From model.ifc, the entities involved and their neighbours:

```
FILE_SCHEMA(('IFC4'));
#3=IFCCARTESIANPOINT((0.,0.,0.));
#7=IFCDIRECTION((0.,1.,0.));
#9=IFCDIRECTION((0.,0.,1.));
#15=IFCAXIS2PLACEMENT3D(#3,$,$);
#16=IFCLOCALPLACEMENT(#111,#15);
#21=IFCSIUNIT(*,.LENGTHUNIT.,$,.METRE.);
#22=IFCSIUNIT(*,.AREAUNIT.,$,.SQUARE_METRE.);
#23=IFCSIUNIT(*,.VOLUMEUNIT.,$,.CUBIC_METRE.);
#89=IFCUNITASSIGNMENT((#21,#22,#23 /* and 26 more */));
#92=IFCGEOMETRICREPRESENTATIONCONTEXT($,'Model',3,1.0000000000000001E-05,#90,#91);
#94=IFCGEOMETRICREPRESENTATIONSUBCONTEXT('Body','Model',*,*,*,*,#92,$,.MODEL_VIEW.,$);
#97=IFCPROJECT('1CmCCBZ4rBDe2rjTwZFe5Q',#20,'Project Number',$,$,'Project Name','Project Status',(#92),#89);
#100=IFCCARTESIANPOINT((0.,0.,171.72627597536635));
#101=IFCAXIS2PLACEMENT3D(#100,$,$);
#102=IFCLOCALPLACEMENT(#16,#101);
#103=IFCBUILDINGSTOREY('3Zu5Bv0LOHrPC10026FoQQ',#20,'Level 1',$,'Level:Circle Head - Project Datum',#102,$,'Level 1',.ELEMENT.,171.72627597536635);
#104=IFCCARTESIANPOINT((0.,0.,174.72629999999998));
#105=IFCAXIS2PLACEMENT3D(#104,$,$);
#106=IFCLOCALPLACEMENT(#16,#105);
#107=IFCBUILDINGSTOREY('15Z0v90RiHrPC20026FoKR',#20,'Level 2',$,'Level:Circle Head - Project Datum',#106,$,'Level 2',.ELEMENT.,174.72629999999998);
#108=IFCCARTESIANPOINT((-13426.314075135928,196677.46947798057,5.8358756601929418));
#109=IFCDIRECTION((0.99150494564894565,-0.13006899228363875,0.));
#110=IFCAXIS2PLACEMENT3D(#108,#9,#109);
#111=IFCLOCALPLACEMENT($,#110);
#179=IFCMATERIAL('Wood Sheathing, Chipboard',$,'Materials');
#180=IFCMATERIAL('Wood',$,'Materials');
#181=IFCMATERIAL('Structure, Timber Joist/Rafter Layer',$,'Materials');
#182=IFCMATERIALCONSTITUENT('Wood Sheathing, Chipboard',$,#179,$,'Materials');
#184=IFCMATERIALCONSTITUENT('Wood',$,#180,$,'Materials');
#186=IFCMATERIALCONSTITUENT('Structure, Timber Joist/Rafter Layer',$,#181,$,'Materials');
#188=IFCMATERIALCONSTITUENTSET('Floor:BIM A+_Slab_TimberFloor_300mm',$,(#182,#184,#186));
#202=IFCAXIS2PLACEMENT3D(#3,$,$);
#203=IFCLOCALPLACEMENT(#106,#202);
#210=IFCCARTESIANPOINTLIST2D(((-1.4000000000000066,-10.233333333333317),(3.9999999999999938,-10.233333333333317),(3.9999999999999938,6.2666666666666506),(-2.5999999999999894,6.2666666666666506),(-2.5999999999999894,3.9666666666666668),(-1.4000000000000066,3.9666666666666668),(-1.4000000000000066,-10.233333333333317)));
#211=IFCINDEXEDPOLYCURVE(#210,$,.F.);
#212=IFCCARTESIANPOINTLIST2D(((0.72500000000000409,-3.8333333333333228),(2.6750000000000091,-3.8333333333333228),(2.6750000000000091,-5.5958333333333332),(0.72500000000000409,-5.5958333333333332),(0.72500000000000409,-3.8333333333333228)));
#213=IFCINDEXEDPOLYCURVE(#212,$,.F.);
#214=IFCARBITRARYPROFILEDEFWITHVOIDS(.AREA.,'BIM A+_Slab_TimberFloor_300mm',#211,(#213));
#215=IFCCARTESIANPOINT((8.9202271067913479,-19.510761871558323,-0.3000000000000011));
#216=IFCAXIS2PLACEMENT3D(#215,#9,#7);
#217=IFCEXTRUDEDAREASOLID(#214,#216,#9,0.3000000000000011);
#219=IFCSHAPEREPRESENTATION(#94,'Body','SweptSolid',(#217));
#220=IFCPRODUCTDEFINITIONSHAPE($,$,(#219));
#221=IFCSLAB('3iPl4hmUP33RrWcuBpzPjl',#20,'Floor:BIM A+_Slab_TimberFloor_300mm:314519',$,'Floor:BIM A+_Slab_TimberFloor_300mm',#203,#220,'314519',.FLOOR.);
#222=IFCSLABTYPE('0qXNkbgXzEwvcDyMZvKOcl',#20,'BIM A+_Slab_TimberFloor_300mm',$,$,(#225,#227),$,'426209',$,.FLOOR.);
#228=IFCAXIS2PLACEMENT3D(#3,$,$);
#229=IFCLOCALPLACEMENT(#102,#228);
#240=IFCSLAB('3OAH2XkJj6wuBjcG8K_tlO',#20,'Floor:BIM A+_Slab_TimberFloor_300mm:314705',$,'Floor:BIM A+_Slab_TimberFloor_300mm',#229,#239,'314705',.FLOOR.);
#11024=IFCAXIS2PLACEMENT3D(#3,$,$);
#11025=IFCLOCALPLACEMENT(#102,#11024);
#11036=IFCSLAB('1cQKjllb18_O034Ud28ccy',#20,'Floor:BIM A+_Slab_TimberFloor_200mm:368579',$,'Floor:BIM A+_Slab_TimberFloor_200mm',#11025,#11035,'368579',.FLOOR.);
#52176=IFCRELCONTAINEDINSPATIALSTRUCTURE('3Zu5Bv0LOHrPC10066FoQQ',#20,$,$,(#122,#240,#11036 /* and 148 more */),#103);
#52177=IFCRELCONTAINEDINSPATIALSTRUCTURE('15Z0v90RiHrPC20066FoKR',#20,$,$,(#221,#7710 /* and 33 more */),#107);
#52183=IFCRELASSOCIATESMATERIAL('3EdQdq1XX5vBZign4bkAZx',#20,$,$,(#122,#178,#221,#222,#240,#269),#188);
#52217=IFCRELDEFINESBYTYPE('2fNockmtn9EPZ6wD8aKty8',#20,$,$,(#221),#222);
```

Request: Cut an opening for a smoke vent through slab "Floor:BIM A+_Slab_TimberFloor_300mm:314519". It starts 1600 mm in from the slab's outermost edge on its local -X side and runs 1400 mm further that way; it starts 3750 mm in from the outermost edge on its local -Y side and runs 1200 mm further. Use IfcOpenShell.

```python
import numpy as np
import ifcopenshell
import ifcopenshell.api.feature
import ifcopenshell.api.geometry
import ifcopenshell.api.root
import ifcopenshell.geom
import ifcopenshell.util.placement
import ifcopenshell.util.representation
import ifcopenshell.util.shape
import ifcopenshell.util.unit

model = ifcopenshell.open("model.ifc")
unit_scale = ifcopenshell.util.unit.calculate_unit_scale(model)
settings = ifcopenshell.geom.settings()


def volume(element):
    """Net volume in cubic metres, openings subtracted."""
    shape = ifcopenshell.geom.create_shape(settings, element)
    return ifcopenshell.util.shape.get_volume(shape.geometry)


slab = model.by_guid("3iPl4hmUP33RrWcuBpzPjl")
before = volume(slab)

# Extent in the slab's own axes, in metres. The edges named are its -X and -Y sides.
slab_shape = ifcopenshell.geom.create_shape(settings, slab)
vertices = ifcopenshell.util.shape.get_vertices(slab_shape.geometry)
x_min, y_min, bottom = vertices.min(axis=0)
top = vertices[:, 2].max()

opening = ifcopenshell.api.root.create_entity(model, ifc_class="IfcOpeningElement", name="Smoke vent opening", predefined_type="OPENING")
context = ifcopenshell.util.representation.get_context(model, "Model", "Body", "MODEL_VIEW")
width, depth = 1.4, 1.2
outline = [(0.0, 0.0), (width, 0.0), (width, depth), (0.0, depth), (0.0, 0.0)]
# Overshoot both faces by 50 mm so the cut is clean.
shape = ifcopenshell.api.geometry.add_slab_representation(
    model, context=context, depth=top - bottom + 0.1, polyline=outline
)
ifcopenshell.api.geometry.assign_representation(model, product=opening, representation=shape)

matrix = ifcopenshell.util.placement.get_local_placement(slab.ObjectPlacement)
matrix[:, 3] = matrix @ np.append(np.array([x_min + 1.6, y_min + 3.75, bottom - 0.05]) / unit_scale, 1.0)
ifcopenshell.api.geometry.edit_object_placement(model, product=opening, matrix=matrix, is_si=False)
ifcopenshell.api.feature.add_feature(model, feature=opening, element=slab)

after = volume(slab)

print(f"slab volume {before:.3f} -> {after:.3f} m3")

model.write("model_rev.ifc")
```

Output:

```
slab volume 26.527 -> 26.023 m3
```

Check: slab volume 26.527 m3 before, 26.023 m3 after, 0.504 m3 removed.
